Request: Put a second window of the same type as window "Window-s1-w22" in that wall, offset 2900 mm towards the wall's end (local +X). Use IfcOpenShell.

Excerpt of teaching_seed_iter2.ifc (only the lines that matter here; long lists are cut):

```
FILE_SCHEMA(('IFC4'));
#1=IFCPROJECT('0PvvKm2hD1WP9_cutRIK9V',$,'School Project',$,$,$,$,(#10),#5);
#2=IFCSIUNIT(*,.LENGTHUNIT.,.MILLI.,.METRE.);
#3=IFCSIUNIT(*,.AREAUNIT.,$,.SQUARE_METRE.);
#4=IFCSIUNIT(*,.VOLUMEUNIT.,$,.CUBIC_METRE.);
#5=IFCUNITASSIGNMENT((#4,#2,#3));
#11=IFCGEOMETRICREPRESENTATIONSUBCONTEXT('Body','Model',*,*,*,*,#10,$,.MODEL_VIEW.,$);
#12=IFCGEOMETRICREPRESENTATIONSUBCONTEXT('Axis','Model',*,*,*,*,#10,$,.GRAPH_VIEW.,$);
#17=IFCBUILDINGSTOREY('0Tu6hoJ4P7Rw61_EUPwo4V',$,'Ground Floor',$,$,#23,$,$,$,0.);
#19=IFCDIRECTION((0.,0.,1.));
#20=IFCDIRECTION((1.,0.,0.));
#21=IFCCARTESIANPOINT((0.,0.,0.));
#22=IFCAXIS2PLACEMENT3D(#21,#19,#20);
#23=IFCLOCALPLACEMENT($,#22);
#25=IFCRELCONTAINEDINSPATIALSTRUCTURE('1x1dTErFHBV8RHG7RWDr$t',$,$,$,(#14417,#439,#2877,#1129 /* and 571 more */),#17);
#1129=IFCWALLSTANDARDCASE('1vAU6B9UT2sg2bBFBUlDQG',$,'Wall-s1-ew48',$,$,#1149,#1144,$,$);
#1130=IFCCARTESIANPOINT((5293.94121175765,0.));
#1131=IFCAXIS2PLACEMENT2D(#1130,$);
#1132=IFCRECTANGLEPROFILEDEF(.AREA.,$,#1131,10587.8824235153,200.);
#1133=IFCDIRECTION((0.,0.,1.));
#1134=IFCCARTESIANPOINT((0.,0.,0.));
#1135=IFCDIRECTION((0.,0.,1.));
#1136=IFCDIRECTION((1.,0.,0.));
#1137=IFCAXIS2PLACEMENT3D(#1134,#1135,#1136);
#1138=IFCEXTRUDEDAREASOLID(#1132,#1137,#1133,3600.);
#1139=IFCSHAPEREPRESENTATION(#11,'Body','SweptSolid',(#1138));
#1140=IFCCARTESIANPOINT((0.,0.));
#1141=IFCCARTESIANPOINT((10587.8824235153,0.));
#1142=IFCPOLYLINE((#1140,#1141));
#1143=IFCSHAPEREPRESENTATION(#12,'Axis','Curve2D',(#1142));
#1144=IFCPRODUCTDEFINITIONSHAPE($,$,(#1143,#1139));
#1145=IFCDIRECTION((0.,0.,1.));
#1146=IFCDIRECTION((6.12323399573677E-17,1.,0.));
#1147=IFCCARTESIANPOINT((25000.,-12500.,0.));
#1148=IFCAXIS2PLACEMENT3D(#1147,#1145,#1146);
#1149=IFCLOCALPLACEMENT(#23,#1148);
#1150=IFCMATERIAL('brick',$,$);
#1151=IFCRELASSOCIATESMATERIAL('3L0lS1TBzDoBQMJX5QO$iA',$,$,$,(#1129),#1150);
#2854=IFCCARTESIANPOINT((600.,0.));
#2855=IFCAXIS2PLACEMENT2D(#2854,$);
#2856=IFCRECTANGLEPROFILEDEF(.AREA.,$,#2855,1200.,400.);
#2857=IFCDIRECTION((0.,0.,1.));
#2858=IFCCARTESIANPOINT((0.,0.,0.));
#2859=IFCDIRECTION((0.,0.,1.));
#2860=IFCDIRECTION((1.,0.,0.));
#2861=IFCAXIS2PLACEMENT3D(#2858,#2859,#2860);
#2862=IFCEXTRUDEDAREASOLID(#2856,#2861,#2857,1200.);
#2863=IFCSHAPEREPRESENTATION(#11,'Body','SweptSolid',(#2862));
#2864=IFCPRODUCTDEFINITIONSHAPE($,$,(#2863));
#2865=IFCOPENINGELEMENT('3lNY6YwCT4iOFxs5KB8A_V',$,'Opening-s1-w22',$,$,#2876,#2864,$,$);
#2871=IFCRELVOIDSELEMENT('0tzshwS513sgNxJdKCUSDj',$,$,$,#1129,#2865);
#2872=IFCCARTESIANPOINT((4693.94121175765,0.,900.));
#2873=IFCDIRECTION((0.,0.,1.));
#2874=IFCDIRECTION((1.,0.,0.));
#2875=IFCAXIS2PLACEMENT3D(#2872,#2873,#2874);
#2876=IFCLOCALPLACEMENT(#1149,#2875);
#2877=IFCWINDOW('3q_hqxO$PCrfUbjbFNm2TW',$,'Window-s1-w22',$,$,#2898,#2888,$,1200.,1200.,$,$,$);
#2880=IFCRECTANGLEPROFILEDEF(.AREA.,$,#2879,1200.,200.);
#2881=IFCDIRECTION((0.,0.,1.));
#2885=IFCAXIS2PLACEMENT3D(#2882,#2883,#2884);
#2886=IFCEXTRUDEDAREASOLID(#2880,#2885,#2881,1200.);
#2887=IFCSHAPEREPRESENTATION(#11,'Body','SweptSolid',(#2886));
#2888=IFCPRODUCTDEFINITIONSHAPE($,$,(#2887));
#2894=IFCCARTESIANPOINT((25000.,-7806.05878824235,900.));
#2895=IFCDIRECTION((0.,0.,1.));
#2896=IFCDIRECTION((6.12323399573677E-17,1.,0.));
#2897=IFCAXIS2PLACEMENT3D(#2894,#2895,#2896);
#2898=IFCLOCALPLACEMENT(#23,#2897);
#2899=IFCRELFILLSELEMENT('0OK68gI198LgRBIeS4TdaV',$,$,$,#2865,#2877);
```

```python
import ifcopenshell
import ifcopenshell.api.feature
import ifcopenshell.api.geometry
import ifcopenshell.api.root
import ifcopenshell.geom
import ifcopenshell.util.element
import ifcopenshell.util.placement
import ifcopenshell.util.shape

model = ifcopenshell.open("teaching_seed_iter2.ifc")
settings = ifcopenshell.geom.settings()


def volume(element):
    """Net volume in cubic metres, openings subtracted."""
    shape = ifcopenshell.geom.create_shape(settings, element)
    return ifcopenshell.util.shape.get_volume(shape.geometry)


window = model.by_guid("3q_hqxO$PCrfUbjbFNm2TW")
opening = window.FillsVoids[0].RelatingOpeningElement
wall = opening.VoidsElements[0].RelatingBuildingElement
before = volume(wall)
shift = ifcopenshell.util.placement.get_local_placement(wall.ObjectPlacement)[:3, 0] * 2900.0

# copy_class copies the void relationship, type, container and properties, but no geometry.
new_opening = ifcopenshell.api.root.copy_class(model, product=opening)
new_opening.Representation = ifcopenshell.util.element.copy_deep(
    model, opening.Representation, exclude=["IfcGeometricRepresentationContext", "IfcRepresentationMap"]
)
new_window = ifcopenshell.api.root.copy_class(model, product=window)
new_window.Representation = ifcopenshell.util.element.copy_deep(
    model, window.Representation, exclude=["IfcGeometricRepresentationContext", "IfcRepresentationMap"]
)
ifcopenshell.api.feature.add_filling(model, opening=new_opening, element=new_window)

for old, new in ((opening, new_opening), (window, new_window)):
    matrix = ifcopenshell.util.placement.get_local_placement(old.ObjectPlacement)
    matrix[:3, 3] += shift
    ifcopenshell.api.geometry.edit_object_placement(model, product=new, matrix=matrix, is_si=False)

after = volume(wall)

print(f"wall volume {before:.3f} -> {after:.3f} m3")

model.write("teaching_seed_iter2-out.ifc")
```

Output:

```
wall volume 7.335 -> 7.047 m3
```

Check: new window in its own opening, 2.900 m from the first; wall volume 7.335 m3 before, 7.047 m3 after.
